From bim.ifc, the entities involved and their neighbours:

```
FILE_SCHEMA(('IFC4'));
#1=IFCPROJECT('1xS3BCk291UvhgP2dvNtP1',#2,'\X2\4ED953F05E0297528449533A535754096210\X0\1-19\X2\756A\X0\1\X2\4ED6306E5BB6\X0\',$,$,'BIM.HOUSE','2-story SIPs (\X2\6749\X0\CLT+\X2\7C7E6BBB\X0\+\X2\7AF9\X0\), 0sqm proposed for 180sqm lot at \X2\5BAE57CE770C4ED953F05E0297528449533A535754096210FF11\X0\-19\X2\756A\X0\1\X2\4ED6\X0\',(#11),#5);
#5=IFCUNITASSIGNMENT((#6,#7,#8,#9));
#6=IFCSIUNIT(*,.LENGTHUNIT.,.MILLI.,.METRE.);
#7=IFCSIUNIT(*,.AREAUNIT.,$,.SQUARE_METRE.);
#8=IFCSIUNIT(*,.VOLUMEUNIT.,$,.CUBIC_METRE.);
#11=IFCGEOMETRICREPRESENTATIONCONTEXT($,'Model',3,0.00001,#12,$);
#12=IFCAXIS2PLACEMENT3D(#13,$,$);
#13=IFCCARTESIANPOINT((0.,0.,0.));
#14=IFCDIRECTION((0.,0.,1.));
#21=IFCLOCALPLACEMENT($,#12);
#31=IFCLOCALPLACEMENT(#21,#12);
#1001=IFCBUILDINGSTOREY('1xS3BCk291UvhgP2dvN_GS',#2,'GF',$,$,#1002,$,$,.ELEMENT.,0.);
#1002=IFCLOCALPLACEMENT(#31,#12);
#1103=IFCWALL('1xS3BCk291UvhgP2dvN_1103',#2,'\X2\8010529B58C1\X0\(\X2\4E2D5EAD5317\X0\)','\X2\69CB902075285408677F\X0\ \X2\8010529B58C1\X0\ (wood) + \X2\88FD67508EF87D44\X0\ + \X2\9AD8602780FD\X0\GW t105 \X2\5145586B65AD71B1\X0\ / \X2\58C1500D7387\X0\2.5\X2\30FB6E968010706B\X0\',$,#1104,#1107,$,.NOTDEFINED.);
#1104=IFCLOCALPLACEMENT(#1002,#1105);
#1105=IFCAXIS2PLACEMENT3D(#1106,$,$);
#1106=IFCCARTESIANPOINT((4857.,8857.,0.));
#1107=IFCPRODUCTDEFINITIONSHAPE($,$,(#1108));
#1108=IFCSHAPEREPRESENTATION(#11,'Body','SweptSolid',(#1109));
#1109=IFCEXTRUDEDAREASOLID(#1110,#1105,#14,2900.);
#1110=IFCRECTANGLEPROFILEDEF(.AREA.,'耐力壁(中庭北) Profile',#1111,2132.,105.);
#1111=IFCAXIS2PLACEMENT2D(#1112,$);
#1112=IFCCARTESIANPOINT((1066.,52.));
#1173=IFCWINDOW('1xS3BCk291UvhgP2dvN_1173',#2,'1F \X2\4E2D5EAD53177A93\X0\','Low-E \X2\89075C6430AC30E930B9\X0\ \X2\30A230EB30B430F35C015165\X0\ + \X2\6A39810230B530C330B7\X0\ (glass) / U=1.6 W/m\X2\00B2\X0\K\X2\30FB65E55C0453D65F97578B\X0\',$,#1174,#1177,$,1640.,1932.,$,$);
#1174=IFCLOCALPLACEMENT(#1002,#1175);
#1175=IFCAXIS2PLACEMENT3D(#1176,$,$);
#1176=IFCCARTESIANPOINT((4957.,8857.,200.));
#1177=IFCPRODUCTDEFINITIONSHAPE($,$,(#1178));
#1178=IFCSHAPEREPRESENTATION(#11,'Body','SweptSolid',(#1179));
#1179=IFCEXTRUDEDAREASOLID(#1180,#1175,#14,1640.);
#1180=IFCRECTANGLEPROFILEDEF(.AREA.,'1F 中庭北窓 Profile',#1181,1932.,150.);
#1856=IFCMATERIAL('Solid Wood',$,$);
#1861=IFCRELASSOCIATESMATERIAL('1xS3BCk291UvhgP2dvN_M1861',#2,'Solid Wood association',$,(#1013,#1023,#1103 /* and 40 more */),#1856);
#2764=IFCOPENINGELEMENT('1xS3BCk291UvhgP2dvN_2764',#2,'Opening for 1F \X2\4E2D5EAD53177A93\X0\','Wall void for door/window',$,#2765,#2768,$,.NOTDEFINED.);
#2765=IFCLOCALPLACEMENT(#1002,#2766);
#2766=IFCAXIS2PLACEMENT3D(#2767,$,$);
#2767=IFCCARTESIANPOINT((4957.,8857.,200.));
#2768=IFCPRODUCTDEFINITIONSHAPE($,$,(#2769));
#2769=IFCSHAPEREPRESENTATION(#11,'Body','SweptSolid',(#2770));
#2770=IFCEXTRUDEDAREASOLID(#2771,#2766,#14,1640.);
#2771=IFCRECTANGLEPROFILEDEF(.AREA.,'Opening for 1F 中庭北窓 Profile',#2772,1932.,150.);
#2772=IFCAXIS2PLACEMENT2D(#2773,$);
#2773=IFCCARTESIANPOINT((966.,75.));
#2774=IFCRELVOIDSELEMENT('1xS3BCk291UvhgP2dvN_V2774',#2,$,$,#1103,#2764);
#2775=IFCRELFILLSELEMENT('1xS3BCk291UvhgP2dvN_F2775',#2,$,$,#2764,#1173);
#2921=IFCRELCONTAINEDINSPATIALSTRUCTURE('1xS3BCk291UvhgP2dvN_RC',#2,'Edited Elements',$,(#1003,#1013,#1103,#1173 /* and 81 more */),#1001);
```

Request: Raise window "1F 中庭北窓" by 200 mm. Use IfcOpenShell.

```python
import numpy as np
import ifcopenshell
import ifcopenshell.api.geometry
import ifcopenshell.util.placement
import ifcopenshell.util.unit

model = ifcopenshell.open("bim.ifc")
unit_scale = ifcopenshell.util.unit.calculate_unit_scale(model)

window = model.by_id(1173)
opening = window.FillsVoids[0].RelatingOpeningElement
dz = 200.0

shift = np.array([0.0, 0.0, dz])
# The window is not placed relative to its opening, so move both.
for product in (opening, window):
    matrix = ifcopenshell.util.placement.get_local_placement(product.ObjectPlacement)
    matrix[:3, 3] += shift
    ifcopenshell.api.geometry.edit_object_placement(model, product=product, matrix=matrix, is_si=False)

print(f"moved by {dz * unit_scale:+.3f} m")

model.write("bim_updated.ifc")
```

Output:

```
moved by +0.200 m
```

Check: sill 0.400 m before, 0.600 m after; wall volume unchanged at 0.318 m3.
